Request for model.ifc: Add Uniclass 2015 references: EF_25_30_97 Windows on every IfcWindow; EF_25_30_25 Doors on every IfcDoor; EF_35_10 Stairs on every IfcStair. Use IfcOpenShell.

First a look at what the model holds.

```python
import ifcopenshell

model = ifcopenshell.open("model.ifc")
print(model.schema)
print("classifications:", [c.Name for c in model.by_type("IfcClassification")])
for ifc_class in ("IfcDoor", "IfcRoof", "IfcStair", "IfcWall", "IfcWindow"):
    print(ifc_class, len(model.by_type(ifc_class)))
```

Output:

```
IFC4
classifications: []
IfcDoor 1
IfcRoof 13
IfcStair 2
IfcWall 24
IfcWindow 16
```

```python
import ifcopenshell
import ifcopenshell.api.classification

model = ifcopenshell.open("model.ifc")

system = ifcopenshell.api.classification.add_classification(model, classification="Uniclass 2015")

codes = {
    "IfcWindow": ("EF_25_30_97", "Windows"),
    "IfcDoor": ("EF_25_30_25", "Doors"),
    "IfcStair": ("EF_35_10", "Stairs"),
}
for ifc_class, (code, name) in codes.items():
    products = model.by_type(ifc_class)
    ifcopenshell.api.classification.add_reference(
        model, products=products, classification=system, identification=code, name=name
    )
    print(code, len(products))

model.write("model-out.ifc")
```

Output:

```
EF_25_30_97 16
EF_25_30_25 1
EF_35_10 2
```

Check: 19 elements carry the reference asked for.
